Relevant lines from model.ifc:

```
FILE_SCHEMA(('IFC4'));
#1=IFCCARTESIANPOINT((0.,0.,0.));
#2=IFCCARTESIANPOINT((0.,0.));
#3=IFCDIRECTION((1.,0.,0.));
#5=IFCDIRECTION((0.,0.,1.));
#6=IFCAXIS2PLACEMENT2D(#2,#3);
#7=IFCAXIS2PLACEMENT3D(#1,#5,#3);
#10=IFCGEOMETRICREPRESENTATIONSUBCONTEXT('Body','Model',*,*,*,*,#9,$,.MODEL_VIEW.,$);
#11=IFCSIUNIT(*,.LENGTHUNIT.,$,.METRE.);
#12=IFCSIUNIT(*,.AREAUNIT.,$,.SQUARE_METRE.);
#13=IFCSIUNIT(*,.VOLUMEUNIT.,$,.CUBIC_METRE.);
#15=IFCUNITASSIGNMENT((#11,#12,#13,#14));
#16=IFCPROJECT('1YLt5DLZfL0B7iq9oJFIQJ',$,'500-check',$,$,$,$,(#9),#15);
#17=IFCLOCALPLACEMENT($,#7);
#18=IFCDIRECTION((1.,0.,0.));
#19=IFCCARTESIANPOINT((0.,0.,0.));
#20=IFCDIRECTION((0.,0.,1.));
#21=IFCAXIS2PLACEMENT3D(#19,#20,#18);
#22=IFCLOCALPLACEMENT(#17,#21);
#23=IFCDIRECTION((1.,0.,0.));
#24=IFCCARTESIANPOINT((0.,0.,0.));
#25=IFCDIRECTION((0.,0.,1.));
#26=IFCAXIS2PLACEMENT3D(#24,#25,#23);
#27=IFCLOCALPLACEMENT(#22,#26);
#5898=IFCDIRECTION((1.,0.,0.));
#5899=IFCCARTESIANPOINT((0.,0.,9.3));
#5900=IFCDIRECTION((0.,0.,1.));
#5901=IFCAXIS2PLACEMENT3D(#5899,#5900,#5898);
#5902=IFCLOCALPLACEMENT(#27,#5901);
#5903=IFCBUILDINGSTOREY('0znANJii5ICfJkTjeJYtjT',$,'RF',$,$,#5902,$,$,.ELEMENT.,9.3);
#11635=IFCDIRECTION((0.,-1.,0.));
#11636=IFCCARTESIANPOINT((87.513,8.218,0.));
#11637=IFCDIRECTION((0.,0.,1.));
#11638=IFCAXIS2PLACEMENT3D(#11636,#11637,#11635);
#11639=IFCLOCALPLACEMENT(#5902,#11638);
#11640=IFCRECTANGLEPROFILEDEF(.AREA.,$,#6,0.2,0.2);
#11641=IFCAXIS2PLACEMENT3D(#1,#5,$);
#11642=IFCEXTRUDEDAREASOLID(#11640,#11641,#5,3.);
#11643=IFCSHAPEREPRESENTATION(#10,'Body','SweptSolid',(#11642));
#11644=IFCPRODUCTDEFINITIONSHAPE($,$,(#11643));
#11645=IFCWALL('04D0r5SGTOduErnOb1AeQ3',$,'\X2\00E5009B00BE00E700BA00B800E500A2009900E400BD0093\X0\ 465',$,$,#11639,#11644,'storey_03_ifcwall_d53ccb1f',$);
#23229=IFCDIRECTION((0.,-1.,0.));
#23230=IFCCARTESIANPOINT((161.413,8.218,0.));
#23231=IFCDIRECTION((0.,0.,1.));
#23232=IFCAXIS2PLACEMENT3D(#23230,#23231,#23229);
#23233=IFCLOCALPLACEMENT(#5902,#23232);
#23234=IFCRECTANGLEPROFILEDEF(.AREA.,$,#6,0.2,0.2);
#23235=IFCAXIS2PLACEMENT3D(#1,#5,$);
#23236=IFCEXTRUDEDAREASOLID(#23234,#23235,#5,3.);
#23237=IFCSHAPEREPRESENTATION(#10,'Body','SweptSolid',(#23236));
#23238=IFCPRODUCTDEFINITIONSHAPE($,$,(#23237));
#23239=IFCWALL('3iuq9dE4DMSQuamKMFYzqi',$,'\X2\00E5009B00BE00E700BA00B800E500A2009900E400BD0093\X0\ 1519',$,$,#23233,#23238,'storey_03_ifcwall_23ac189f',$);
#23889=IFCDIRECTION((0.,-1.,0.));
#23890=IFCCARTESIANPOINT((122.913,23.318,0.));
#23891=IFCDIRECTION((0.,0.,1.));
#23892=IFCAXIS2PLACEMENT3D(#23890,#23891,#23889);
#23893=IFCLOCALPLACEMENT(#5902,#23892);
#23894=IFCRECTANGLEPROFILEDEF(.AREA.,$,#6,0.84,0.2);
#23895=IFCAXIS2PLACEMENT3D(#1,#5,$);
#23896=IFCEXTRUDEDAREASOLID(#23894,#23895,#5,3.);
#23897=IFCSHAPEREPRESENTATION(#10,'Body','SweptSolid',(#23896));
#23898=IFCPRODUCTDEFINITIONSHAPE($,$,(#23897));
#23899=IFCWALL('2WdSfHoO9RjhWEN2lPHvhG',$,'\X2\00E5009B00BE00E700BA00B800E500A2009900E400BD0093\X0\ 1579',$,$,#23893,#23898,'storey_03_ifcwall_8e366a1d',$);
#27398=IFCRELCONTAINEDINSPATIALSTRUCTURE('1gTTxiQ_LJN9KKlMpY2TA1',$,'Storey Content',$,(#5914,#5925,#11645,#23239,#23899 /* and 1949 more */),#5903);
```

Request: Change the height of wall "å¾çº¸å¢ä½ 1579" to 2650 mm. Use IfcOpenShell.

```python
import ifcopenshell
import ifcopenshell.geom
import ifcopenshell.util.representation
import ifcopenshell.util.shape
import ifcopenshell.util.unit

model = ifcopenshell.open("model.ifc")
unit_scale = ifcopenshell.util.unit.calculate_unit_scale(model)
settings = ifcopenshell.geom.settings()


def volume(element):
    """Net volume in cubic metres, openings subtracted."""
    shape = ifcopenshell.geom.create_shape(settings, element)
    return ifcopenshell.util.shape.get_volume(shape.geometry)


wall = model.by_guid("2WdSfHoO9RjhWEN2lPHvhG")
before = volume(wall)

body = ifcopenshell.util.representation.get_representation(wall, "Model", "Body")
solid = body.Items[0]
old_height = solid.Depth
solid.Depth = 2.65 / unit_scale
after = volume(wall)

print(f"height {old_height:g} -> {solid.Depth:g}, volume {before:.3f} -> {after:.3f} m3")

model.write("model_rev.ifc")
```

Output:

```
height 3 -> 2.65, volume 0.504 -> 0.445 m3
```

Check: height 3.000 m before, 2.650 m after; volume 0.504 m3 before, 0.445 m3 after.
